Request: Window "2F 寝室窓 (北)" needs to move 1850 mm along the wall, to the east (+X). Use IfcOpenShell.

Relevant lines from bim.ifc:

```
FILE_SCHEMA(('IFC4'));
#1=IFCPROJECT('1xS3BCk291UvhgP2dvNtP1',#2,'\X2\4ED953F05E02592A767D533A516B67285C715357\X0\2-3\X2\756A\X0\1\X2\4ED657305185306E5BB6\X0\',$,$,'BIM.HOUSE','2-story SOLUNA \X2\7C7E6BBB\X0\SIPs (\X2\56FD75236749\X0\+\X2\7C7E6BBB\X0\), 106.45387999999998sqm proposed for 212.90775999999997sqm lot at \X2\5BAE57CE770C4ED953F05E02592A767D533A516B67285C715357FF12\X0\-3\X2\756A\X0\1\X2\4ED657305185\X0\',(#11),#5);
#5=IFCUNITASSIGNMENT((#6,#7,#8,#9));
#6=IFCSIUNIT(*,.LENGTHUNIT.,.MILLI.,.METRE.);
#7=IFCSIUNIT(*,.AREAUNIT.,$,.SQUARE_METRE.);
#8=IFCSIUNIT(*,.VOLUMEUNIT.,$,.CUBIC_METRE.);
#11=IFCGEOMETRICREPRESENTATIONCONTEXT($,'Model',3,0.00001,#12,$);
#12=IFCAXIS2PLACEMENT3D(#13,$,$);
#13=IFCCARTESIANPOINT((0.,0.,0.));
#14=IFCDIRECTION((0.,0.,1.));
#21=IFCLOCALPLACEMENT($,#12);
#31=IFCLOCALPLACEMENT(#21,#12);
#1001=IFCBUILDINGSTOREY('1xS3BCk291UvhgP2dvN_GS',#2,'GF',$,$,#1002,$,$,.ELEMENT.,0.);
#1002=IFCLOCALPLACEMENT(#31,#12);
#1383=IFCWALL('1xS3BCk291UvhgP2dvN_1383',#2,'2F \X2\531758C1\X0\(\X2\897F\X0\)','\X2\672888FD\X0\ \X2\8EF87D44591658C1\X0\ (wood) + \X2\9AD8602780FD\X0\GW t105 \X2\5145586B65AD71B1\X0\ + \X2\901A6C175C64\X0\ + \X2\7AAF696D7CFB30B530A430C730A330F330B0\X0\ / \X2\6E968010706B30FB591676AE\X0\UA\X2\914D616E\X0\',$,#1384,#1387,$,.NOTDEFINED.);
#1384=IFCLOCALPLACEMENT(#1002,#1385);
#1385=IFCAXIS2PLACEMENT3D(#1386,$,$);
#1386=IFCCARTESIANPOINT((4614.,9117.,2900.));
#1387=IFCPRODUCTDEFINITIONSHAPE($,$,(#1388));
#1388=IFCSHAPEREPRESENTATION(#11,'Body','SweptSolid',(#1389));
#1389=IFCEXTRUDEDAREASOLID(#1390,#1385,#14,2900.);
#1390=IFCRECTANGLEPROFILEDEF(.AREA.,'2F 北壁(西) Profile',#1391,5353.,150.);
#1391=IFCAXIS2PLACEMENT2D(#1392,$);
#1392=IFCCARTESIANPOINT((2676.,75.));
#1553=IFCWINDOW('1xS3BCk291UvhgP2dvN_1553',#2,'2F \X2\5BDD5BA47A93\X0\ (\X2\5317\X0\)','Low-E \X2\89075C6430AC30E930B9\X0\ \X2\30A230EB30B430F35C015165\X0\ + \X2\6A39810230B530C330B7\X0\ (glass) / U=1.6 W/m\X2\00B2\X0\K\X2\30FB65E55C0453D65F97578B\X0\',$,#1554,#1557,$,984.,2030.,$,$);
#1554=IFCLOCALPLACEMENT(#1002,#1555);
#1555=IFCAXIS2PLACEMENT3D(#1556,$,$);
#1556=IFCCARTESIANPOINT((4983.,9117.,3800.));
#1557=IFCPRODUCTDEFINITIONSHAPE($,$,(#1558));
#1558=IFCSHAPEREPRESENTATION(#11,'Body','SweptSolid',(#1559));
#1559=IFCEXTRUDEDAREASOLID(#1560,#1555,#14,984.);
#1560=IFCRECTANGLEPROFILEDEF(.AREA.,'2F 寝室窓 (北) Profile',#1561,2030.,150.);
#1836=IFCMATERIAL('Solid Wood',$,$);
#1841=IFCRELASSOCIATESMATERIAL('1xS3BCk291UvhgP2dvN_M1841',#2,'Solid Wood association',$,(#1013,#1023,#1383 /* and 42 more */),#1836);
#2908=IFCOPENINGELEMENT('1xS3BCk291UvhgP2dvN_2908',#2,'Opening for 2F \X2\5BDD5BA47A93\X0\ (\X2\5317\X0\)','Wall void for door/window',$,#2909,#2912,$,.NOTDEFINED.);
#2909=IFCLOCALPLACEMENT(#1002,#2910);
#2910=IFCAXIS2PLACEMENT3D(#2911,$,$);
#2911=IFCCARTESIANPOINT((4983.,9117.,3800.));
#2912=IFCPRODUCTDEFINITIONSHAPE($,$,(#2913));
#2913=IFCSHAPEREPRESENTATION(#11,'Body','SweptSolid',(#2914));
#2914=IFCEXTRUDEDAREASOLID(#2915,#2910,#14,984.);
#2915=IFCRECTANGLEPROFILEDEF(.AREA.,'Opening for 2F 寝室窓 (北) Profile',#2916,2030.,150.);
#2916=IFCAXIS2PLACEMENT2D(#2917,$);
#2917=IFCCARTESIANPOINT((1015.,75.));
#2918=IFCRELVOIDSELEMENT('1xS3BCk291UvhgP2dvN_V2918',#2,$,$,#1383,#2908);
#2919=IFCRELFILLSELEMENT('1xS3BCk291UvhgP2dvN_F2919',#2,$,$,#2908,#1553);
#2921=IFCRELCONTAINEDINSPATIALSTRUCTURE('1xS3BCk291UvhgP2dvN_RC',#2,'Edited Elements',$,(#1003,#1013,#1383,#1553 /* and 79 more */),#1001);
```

```python
import ifcopenshell
import ifcopenshell.api.geometry
import ifcopenshell.util.placement

model = ifcopenshell.open("bim.ifc")

window = model.by_id(1553)
opening = window.FillsVoids[0].RelatingOpeningElement
wall = opening.VoidsElements[0].RelatingBuildingElement

wall_matrix = ifcopenshell.util.placement.get_local_placement(wall.ObjectPlacement)
shift = wall_matrix[:3, 0] * 1850.0
before = ifcopenshell.util.placement.get_local_placement(window.ObjectPlacement)[:3, 3].copy()

# The window is not placed relative to its opening, so move both.
for product in (opening, window):
    matrix = ifcopenshell.util.placement.get_local_placement(product.ObjectPlacement)
    matrix[:3, 3] += shift
    ifcopenshell.api.geometry.edit_object_placement(model, product=product, matrix=matrix, is_si=False)

after = ifcopenshell.util.placement.get_local_placement(window.ObjectPlacement)[:3, 3]
print("window moved by", (after - before).round(3) + 0.0)

model.write("bim_rev.ifc")
```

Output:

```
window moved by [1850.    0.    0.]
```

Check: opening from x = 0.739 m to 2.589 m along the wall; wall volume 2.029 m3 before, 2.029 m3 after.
